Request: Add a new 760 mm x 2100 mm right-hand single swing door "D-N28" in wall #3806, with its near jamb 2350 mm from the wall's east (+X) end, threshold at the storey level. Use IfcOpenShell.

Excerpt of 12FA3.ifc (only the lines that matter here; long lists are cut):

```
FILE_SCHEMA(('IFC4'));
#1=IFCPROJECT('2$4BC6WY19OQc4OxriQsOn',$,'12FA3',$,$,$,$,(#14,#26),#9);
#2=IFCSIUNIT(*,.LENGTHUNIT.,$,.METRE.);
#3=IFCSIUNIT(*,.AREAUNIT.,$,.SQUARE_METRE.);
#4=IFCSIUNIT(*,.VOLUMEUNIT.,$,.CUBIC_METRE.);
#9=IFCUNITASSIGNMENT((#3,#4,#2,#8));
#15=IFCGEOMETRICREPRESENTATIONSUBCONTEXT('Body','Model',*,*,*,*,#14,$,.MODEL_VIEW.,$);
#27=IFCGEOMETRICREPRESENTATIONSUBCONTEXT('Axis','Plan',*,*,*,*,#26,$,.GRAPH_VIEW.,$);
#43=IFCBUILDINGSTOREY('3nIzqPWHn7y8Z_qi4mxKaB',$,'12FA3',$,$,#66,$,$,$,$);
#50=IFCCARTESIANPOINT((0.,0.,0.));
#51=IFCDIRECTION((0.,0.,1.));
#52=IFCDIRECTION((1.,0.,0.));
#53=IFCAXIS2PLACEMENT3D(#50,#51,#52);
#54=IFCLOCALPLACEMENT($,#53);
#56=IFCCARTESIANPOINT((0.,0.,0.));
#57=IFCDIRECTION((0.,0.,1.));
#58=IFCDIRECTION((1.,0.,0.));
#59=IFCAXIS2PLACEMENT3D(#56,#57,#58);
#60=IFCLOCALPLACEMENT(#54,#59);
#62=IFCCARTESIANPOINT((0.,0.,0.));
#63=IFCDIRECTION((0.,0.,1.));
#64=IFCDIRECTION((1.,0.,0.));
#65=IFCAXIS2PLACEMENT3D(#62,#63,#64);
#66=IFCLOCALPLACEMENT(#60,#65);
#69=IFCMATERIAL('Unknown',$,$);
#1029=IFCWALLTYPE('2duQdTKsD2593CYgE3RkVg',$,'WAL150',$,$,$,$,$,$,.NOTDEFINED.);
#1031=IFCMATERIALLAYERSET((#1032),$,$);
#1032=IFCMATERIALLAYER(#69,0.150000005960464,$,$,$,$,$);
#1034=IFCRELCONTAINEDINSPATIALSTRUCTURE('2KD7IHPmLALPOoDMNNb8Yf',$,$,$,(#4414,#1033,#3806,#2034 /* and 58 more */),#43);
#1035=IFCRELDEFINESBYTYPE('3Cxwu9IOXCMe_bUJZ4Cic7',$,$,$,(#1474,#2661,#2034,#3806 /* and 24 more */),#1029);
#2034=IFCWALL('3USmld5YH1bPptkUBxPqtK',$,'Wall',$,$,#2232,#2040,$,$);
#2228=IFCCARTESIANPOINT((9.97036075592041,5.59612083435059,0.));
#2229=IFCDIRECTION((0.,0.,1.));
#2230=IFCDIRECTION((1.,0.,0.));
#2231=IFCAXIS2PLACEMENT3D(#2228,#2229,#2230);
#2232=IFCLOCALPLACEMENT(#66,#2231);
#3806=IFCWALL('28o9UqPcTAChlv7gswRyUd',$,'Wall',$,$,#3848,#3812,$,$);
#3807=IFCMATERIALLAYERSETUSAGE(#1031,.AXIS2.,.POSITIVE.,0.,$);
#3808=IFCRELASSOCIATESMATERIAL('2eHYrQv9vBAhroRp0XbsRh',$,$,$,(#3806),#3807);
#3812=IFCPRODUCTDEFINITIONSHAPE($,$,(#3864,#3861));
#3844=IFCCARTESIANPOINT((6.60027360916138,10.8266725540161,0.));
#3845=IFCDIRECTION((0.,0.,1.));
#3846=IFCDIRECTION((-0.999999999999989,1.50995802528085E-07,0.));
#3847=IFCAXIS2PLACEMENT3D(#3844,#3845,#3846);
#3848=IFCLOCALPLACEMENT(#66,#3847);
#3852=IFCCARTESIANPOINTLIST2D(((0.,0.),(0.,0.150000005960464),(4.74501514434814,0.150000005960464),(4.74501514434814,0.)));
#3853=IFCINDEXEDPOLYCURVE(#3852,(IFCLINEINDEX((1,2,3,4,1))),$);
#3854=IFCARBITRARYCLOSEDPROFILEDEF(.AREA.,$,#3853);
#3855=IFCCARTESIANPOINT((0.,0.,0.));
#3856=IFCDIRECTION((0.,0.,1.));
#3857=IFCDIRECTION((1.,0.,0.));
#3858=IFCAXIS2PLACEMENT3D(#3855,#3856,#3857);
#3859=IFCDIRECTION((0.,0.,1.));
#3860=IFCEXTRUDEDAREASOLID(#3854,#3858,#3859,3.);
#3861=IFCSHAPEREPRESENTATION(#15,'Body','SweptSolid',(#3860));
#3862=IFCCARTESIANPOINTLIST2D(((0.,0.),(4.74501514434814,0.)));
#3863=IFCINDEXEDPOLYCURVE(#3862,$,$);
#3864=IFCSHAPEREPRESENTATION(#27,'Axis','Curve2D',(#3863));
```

```python
import numpy as np
import ifcopenshell
import ifcopenshell.api.feature
import ifcopenshell.api.geometry
import ifcopenshell.api.root
import ifcopenshell.api.spatial
import ifcopenshell.geom
import ifcopenshell.util.element
import ifcopenshell.util.placement
import ifcopenshell.util.representation
import ifcopenshell.util.shape
import ifcopenshell.util.unit

model = ifcopenshell.open("12FA3.ifc")
unit_scale = ifcopenshell.util.unit.calculate_unit_scale(model)
settings = ifcopenshell.geom.settings()


def volume(element):
    """Net volume in cubic metres, openings subtracted."""
    shape = ifcopenshell.geom.create_shape(settings, element)
    return ifcopenshell.util.shape.get_volume(shape.geometry)


wall = model.by_id(3806)
storey = ifcopenshell.util.element.get_container(wall, ifc_class="IfcBuildingStorey")
context = ifcopenshell.util.representation.get_context(model, "Model", "Body", "MODEL_VIEW")
before = volume(wall)

width, height, from_end, sill = 0.76, 2.1, 2.35, 0.0  # metres

# The wall runs along its own X axis, and the end named is its -X end.
wall_shape = ifcopenshell.geom.create_shape(settings, wall)
x, y, z = ifcopenshell.util.shape.get_vertices(wall_shape.geometry).T
start = x.min() + from_end
face, thickness = float(y.min()), float(y.max() - y.min())
wall_matrix = ifcopenshell.util.placement.get_local_placement(wall.ObjectPlacement)
level = ifcopenshell.util.placement.get_local_placement(storey.ObjectPlacement)[2, 3]


def in_wall(x, y):
    """Placement at x, y metres in the wall's axes, at sill height."""
    matrix = wall_matrix.copy()
    matrix[:, 3] = wall_matrix @ np.array([x / unit_scale, y / unit_scale, 0.0, 1.0])
    matrix[2, 3] = level + sill / unit_scale
    return matrix


# Opening: a box that overshoots both wall faces by 50 mm.
opening = ifcopenshell.api.root.create_entity(model, ifc_class="IfcOpeningElement", predefined_type="OPENING")
box = ifcopenshell.api.geometry.add_wall_representation(
    model, context=context, length=width, height=height, thickness=thickness + 0.1
)
ifcopenshell.api.geometry.assign_representation(model, product=opening, representation=box)
ifcopenshell.api.geometry.edit_object_placement(model, product=opening, matrix=in_wall(start, face - 0.05), is_si=False)
ifcopenshell.api.feature.add_feature(model, feature=opening, element=wall)

door = ifcopenshell.api.root.create_entity(model, ifc_class="IfcDoor", name="D-N28", predefined_type="DOOR")
door.OverallWidth, door.OverallHeight = width / unit_scale, height / unit_scale
door.OperationType = "SINGLE_SWING_RIGHT"
body = ifcopenshell.api.geometry.add_door_representation(
    model,
    context=context,
    overall_width=door.OverallWidth,
    overall_height=door.OverallHeight,
    operation_type="SINGLE_SWING_RIGHT",
    lining_properties={"LiningDepth": thickness / unit_scale, "ThresholdDepth": thickness / unit_scale},
)
ifcopenshell.api.geometry.assign_representation(model, product=door, representation=body)
ifcopenshell.api.spatial.assign_container(model, products=[door], relating_structure=storey)
ifcopenshell.api.feature.add_filling(model, opening=opening, element=door)

# The lining spans the wall, so the door starts at the wall face.
ifcopenshell.api.geometry.edit_object_placement(model, product=door, matrix=in_wall(start, face), is_si=False)

after = volume(wall)

print(f"wall volume {before:.3f} -> {after:.3f} m3")

model.write("12FA3-out.ifc")
```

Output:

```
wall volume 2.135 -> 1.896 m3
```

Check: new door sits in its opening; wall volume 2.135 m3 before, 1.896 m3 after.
